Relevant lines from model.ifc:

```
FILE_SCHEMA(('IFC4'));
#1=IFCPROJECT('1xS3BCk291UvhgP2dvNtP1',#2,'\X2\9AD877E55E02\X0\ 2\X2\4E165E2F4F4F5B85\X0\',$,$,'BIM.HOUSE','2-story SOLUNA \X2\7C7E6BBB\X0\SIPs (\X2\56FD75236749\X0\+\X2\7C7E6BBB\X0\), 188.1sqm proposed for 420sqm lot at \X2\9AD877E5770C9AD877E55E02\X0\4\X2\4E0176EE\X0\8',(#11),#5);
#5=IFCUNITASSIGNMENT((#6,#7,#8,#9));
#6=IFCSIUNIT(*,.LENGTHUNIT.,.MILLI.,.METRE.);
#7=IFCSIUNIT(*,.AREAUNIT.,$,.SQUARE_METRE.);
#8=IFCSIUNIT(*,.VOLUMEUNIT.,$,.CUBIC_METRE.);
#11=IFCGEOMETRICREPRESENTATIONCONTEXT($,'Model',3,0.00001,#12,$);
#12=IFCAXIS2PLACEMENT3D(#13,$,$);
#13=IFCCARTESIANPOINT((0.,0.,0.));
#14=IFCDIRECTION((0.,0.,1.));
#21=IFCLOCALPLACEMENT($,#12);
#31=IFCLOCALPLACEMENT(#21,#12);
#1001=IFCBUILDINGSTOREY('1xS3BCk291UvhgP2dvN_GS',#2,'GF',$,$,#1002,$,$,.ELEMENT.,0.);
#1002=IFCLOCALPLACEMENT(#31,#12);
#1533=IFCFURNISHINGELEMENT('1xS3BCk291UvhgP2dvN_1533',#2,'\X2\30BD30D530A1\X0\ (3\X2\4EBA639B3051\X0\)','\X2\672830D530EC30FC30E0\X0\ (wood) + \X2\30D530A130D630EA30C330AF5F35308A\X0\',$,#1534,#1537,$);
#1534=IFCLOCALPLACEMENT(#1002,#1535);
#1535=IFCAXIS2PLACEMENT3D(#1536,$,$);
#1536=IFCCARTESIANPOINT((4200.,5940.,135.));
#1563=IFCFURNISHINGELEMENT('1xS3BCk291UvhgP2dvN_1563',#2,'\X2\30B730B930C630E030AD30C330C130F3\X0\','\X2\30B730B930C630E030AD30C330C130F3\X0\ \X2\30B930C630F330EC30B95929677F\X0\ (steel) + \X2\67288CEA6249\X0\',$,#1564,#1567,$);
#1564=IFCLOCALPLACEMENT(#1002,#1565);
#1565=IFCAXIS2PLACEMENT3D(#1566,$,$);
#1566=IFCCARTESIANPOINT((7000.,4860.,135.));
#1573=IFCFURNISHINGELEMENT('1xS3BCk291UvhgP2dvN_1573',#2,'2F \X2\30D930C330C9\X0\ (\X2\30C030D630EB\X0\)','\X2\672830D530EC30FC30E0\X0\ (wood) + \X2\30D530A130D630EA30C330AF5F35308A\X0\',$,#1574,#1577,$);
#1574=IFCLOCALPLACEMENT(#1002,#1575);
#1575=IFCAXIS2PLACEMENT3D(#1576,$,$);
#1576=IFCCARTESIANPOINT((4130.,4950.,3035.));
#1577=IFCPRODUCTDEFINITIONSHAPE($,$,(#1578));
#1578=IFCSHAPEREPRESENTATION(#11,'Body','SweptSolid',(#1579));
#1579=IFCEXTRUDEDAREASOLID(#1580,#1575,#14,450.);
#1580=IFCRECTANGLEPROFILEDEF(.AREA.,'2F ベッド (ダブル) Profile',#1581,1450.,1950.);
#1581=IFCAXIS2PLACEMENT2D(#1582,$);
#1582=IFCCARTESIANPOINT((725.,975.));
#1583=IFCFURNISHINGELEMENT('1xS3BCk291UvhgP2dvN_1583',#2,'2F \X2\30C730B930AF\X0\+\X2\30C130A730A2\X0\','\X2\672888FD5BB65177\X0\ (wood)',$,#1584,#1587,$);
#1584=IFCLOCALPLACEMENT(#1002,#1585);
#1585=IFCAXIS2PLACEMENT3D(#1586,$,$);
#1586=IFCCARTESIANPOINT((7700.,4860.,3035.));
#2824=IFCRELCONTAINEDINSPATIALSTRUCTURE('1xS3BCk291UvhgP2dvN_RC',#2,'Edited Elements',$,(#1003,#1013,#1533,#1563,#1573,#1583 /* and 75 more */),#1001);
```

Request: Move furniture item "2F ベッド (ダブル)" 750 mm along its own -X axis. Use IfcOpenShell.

```python
import ifcopenshell
import ifcopenshell.api.geometry
import ifcopenshell.util.placement
import ifcopenshell.util.unit

model = ifcopenshell.open("model.ifc")
unit_scale = ifcopenshell.util.unit.calculate_unit_scale(model)

item = model.by_id(1573)
matrix = ifcopenshell.util.placement.get_local_placement(item.ObjectPlacement)
matrix[:3, 3] -= matrix[:3, 0] * 0.75 / unit_scale
ifcopenshell.api.geometry.edit_object_placement(model, product=item, matrix=matrix, is_si=False)

print(ifcopenshell.util.placement.get_local_placement(item.ObjectPlacement).round(3) + 0.0)

model.write("model_rev.ifc")
```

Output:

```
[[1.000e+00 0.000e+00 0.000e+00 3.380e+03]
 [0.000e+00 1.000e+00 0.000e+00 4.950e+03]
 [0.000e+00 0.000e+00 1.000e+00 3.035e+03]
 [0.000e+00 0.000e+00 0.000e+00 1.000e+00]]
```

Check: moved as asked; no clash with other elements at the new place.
